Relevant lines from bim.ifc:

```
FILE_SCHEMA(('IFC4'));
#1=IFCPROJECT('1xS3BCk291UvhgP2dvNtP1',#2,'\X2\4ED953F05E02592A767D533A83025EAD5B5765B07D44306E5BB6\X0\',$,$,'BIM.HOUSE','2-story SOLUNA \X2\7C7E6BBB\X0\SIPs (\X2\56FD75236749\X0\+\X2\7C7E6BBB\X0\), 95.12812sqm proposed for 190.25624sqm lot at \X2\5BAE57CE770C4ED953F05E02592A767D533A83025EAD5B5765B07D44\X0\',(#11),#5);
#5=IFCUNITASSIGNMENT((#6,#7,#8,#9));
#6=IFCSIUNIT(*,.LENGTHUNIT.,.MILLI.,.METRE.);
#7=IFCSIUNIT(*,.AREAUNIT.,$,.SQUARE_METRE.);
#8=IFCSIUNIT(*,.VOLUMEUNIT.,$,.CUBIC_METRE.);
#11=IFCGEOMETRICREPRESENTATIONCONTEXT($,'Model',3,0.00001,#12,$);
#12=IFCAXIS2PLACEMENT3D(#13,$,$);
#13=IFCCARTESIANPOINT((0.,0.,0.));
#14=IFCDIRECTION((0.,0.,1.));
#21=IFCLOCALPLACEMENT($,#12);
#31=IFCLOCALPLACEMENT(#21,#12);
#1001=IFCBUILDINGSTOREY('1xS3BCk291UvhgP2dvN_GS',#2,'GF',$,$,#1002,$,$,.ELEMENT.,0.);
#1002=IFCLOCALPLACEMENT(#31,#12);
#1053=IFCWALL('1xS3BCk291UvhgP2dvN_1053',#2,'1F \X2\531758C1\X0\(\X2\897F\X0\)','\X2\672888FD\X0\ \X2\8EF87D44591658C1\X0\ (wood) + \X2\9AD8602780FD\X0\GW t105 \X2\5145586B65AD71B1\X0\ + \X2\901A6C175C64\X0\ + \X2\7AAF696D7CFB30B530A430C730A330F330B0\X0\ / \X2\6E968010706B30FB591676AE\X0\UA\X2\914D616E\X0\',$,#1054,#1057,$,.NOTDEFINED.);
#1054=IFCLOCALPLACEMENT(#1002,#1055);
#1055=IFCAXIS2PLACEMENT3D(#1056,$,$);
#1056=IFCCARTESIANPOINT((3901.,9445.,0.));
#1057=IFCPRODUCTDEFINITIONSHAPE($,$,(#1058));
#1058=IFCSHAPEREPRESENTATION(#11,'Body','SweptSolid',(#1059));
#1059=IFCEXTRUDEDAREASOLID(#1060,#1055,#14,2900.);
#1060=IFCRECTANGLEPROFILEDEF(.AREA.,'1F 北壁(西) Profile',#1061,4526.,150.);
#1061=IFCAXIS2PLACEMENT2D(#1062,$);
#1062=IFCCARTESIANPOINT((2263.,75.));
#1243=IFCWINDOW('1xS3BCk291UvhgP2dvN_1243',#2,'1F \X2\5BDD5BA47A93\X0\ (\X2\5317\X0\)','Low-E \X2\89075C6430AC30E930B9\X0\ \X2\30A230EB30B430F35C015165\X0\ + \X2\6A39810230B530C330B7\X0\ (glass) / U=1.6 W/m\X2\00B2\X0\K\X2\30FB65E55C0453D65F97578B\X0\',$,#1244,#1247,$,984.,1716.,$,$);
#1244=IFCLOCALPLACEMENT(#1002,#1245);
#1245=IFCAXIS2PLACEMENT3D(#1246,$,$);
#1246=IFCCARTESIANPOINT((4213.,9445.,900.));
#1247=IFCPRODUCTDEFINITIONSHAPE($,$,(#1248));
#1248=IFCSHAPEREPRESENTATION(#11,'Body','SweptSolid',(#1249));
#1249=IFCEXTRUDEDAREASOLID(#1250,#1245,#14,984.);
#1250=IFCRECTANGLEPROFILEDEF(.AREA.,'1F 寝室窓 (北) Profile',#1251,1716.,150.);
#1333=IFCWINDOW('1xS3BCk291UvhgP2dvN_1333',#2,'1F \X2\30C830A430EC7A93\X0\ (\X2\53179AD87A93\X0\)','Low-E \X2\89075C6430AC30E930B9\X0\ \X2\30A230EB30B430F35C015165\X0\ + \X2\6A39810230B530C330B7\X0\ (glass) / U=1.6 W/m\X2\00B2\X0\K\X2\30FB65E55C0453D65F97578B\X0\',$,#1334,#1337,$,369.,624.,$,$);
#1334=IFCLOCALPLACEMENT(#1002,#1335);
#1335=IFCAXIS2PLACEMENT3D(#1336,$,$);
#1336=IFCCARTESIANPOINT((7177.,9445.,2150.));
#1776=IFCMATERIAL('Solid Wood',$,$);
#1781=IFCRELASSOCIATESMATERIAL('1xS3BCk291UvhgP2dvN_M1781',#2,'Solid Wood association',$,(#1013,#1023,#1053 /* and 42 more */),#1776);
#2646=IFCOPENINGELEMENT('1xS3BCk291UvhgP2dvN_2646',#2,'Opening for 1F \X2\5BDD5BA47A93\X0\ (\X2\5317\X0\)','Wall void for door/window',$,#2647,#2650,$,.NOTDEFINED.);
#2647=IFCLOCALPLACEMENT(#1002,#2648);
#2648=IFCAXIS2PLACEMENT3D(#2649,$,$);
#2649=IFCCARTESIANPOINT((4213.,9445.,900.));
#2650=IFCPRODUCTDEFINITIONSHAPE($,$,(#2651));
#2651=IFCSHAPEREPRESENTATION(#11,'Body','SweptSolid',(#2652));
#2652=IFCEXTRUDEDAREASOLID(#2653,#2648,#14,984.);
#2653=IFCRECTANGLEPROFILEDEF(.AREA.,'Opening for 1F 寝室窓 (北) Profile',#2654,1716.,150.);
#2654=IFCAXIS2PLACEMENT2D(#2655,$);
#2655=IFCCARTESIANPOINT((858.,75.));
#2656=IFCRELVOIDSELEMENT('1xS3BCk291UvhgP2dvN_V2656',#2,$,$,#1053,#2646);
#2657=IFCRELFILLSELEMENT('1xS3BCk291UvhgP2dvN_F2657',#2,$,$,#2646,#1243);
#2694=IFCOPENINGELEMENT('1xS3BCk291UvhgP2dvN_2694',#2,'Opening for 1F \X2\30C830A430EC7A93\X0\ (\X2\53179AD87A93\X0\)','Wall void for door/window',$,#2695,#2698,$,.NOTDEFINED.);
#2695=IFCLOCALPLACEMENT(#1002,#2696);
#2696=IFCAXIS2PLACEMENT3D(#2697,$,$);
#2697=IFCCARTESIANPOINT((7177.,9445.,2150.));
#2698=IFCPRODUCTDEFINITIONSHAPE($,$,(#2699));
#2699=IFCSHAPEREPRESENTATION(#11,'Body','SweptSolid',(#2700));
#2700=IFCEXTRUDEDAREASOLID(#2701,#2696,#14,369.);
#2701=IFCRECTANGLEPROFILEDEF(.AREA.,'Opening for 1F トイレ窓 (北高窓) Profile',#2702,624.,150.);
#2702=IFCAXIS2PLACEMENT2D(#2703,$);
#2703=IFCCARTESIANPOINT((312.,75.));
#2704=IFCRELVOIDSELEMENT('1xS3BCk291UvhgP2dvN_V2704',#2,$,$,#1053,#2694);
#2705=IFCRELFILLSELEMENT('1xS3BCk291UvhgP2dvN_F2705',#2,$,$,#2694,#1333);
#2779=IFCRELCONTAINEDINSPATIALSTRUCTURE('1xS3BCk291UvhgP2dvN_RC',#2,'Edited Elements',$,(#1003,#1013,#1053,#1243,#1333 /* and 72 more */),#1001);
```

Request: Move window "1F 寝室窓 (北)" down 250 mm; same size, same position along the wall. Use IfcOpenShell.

```python
import numpy as np
import ifcopenshell
import ifcopenshell.api.geometry
import ifcopenshell.util.placement
import ifcopenshell.util.unit

model = ifcopenshell.open("bim.ifc")
unit_scale = ifcopenshell.util.unit.calculate_unit_scale(model)

window = model.by_guid("1xS3BCk291UvhgP2dvN_1243")
opening = window.FillsVoids[0].RelatingOpeningElement
dz = -250.0

shift = np.array([0.0, 0.0, dz])
# The window is not placed relative to its opening, so move both.
for product in (opening, window):
    matrix = ifcopenshell.util.placement.get_local_placement(product.ObjectPlacement)
    matrix[:3, 3] += shift
    ifcopenshell.api.geometry.edit_object_placement(model, product=product, matrix=matrix, is_si=False)

print(f"moved by {dz * unit_scale:+.3f} m")

model.write("bim_edited.ifc")
```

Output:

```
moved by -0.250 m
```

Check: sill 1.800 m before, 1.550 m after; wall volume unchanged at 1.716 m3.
